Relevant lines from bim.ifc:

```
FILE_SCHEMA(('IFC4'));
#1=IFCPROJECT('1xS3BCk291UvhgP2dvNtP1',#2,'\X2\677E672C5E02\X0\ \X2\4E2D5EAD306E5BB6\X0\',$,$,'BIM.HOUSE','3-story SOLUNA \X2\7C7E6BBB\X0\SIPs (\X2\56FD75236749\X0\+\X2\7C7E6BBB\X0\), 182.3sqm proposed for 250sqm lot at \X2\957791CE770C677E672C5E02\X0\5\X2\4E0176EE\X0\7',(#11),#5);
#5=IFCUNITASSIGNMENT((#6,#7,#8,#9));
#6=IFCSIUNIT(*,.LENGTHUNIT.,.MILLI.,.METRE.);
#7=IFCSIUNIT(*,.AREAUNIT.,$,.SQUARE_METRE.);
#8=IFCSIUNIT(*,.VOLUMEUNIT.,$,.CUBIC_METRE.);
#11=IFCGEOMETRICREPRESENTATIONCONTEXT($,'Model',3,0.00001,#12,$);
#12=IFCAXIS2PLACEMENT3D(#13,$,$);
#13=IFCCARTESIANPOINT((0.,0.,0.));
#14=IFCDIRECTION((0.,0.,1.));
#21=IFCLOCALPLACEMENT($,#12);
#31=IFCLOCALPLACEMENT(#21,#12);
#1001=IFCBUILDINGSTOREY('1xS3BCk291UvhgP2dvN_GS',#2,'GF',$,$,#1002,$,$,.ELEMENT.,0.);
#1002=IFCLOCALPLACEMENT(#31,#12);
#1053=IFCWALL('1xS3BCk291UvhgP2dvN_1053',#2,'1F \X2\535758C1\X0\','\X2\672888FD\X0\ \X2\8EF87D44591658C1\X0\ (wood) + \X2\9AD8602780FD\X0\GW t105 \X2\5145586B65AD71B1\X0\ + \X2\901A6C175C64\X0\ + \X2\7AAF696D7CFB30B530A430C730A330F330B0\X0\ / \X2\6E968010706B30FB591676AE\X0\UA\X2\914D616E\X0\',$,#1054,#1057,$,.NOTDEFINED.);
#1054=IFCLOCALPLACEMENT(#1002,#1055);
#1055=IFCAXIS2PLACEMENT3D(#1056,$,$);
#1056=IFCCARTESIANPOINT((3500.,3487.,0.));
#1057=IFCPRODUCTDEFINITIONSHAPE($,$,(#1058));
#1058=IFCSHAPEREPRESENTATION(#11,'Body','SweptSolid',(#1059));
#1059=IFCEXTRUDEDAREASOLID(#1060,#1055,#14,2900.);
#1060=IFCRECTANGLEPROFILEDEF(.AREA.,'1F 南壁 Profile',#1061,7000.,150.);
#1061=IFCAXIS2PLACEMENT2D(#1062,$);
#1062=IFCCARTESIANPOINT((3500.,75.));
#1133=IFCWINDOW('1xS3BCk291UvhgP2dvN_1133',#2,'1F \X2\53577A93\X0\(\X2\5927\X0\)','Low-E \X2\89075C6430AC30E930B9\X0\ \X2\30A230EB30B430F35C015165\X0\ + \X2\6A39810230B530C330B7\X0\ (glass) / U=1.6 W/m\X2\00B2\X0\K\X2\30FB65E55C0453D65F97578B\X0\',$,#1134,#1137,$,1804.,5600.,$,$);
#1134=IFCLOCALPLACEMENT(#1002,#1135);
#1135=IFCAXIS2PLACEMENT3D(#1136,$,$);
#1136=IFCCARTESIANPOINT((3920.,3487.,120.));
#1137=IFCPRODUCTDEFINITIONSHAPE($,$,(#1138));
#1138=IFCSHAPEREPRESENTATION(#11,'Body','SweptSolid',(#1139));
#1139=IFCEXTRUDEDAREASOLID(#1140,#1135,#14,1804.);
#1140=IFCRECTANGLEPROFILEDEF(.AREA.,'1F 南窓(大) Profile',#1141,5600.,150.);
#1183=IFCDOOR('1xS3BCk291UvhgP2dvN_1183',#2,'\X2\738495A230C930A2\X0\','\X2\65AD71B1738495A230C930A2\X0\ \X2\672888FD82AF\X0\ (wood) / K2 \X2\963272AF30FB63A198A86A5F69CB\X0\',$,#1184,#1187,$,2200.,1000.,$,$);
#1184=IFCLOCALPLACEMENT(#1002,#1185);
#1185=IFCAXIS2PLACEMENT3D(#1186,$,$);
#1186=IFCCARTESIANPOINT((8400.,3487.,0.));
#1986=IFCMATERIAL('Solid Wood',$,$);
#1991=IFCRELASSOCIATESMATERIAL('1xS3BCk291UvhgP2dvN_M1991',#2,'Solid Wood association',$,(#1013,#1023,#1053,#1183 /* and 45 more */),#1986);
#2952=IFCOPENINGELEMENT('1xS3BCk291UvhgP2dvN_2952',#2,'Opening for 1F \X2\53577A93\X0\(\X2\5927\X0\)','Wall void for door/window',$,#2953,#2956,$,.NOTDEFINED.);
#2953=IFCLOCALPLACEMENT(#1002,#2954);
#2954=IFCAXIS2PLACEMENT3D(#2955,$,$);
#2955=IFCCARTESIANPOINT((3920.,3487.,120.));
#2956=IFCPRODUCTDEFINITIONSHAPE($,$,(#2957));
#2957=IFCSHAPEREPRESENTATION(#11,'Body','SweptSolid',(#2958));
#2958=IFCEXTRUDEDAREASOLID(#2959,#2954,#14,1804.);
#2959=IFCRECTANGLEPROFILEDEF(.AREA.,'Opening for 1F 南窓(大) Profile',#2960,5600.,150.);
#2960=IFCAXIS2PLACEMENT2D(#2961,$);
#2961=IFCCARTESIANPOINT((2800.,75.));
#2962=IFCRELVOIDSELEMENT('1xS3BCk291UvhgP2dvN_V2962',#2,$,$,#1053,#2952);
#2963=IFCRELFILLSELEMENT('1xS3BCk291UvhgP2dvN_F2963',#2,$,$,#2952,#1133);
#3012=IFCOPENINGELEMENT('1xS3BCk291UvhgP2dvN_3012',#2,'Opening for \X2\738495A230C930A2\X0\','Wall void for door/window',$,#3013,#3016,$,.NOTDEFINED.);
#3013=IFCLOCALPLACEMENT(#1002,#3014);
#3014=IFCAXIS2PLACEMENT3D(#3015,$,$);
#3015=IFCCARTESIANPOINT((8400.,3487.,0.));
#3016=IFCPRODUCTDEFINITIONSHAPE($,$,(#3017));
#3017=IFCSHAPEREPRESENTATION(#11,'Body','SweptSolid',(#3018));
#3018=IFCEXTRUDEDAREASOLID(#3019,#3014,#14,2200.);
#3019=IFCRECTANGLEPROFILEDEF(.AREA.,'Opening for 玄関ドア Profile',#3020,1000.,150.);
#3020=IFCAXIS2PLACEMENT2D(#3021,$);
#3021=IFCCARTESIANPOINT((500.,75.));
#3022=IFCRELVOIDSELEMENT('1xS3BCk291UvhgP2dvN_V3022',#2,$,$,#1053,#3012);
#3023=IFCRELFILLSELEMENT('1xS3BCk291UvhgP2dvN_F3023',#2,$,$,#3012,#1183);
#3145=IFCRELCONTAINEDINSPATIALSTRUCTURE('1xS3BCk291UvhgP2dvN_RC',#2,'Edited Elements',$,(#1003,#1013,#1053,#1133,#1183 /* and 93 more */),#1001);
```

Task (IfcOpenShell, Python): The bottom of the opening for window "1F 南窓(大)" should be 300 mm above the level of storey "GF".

```python
import numpy as np
import ifcopenshell
import ifcopenshell.api.geometry
import ifcopenshell.geom
import ifcopenshell.util.element
import ifcopenshell.util.placement
import ifcopenshell.util.shape
import ifcopenshell.util.unit

model = ifcopenshell.open("bim.ifc")
unit_scale = ifcopenshell.util.unit.calculate_unit_scale(model)

window = model.by_id(1133)
opening = window.FillsVoids[0].RelatingOpeningElement
storey = ifcopenshell.util.element.get_container(window, ifc_class="IfcBuildingStorey")
level = ifcopenshell.util.placement.get_local_placement(storey.ObjectPlacement)[2, 3]

# The opening's origin need not be at the sill, so measure its lowest point.
shape = ifcopenshell.geom.create_shape(ifcopenshell.geom.settings(), opening)
bottom = ifcopenshell.util.shape.get_shape_bottom_elevation(shape, shape.geometry) / unit_scale
dz = level + 0.3 / unit_scale - bottom

shift = np.array([0.0, 0.0, dz])
# The window is not placed relative to its opening, so move both.
for product in (opening, window):
    matrix = ifcopenshell.util.placement.get_local_placement(product.ObjectPlacement)
    matrix[:3, 3] += shift
    ifcopenshell.api.geometry.edit_object_placement(model, product=product, matrix=matrix, is_si=False)

print(f"moved by {dz * unit_scale:+.3f} m")

model.write("bim_edited.ifc")
```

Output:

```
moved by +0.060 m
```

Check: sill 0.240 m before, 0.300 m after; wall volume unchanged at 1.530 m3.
